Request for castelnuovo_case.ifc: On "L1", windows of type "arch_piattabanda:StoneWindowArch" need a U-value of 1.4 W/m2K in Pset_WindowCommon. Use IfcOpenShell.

First a look at what the model holds.

```python
import ifcopenshell
import ifcopenshell.util.element

model = ifcopenshell.open("castelnuovo_case.ifc")
print(model.schema)
storey = next(s for s in model.by_type("IfcBuildingStorey") if s.Name == "L1")
windows = [e for e in ifcopenshell.util.element.get_decomposition(storey) if e.is_a("IfcWindow")]
seen = {}
for e in windows:
    element_type = ifcopenshell.util.element.get_type(e)
    key = (element_type.Name if element_type != e and element_type else None, ifcopenshell.util.element.get_pset(e, "Pset_WindowCommon", "ThermalTransmittance"))
    seen[key] = seen.get(key, 0) + 1
for (name, value), count in sorted(seen.items(), key=str):
    print(count, "x", name, "|", value)
```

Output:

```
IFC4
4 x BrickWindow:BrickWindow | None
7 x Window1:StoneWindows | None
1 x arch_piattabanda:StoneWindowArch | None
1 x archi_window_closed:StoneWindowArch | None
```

```python
import ifcopenshell
import ifcopenshell.api.pset
import ifcopenshell.util.element

model = ifcopenshell.open("castelnuovo_case.ifc")

storey = next(s for s in model.by_type("IfcBuildingStorey") if s.Name == "L1")
windows = [e for e in ifcopenshell.util.element.get_decomposition(storey) if e.is_a("IfcWindow")]

count = 0
for e in windows:
    element_type = ifcopenshell.util.element.get_type(e)
    if element_type in (None, e) or element_type.Name != "arch_piattabanda:StoneWindowArch":
        continue
    # add_pset returns the element's existing set when there is one.
    pset = ifcopenshell.api.pset.add_pset(model, product=e, name="Pset_WindowCommon")
    ifcopenshell.api.pset.edit_pset(model, pset=pset, properties={"ThermalTransmittance": 1.4})
    count += 1

print(count, "windows updated")

model.write("castelnuovo_case_v2.ifc")
```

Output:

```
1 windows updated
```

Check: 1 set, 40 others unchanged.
